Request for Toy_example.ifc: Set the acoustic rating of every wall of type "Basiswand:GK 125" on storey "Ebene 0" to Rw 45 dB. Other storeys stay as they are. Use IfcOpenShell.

First a look at what the model holds.

```python
import ifcopenshell
import ifcopenshell.util.element

model = ifcopenshell.open("Toy_example.ifc")
print(model.schema)
storey = next(s for s in model.by_type("IfcBuildingStorey") if s.Name == "Ebene 0")
walls = [e for e in ifcopenshell.util.element.get_decomposition(storey) if e.is_a("IfcWall")]
seen = {}
for e in walls:
    element_type = ifcopenshell.util.element.get_type(e)
    key = (element_type.Name if element_type != e and element_type else None, ifcopenshell.util.element.get_pset(e, "Pset_WallCommon", "AcousticRating"))
    seen[key] = seen.get(key, 0) + 1
for (name, value), count in sorted(seen.items(), key=str):
    print(count, "x", name, "|", value)
```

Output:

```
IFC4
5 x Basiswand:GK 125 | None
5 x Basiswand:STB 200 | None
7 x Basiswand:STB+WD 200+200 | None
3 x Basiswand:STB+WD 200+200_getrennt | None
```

```python
import ifcopenshell
import ifcopenshell.api.pset
import ifcopenshell.util.element

model = ifcopenshell.open("Toy_example.ifc")

storey = next(s for s in model.by_type("IfcBuildingStorey") if s.Name == "Ebene 0")
walls = [e for e in ifcopenshell.util.element.get_decomposition(storey) if e.is_a("IfcWall")]

count = 0
for e in walls:
    element_type = ifcopenshell.util.element.get_type(e)
    if element_type in (None, e) or element_type.Name != "Basiswand:GK 125":
        continue
    # add_pset returns the element's existing set when there is one.
    pset = ifcopenshell.api.pset.add_pset(model, product=e, name="Pset_WallCommon")
    ifcopenshell.api.pset.edit_pset(model, pset=pset, properties={"AcousticRating": "Rw 45 dB"})
    count += 1

print(count, "walls updated")

model.write("Toy_example_rev.ifc")
```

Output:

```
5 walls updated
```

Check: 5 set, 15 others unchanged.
